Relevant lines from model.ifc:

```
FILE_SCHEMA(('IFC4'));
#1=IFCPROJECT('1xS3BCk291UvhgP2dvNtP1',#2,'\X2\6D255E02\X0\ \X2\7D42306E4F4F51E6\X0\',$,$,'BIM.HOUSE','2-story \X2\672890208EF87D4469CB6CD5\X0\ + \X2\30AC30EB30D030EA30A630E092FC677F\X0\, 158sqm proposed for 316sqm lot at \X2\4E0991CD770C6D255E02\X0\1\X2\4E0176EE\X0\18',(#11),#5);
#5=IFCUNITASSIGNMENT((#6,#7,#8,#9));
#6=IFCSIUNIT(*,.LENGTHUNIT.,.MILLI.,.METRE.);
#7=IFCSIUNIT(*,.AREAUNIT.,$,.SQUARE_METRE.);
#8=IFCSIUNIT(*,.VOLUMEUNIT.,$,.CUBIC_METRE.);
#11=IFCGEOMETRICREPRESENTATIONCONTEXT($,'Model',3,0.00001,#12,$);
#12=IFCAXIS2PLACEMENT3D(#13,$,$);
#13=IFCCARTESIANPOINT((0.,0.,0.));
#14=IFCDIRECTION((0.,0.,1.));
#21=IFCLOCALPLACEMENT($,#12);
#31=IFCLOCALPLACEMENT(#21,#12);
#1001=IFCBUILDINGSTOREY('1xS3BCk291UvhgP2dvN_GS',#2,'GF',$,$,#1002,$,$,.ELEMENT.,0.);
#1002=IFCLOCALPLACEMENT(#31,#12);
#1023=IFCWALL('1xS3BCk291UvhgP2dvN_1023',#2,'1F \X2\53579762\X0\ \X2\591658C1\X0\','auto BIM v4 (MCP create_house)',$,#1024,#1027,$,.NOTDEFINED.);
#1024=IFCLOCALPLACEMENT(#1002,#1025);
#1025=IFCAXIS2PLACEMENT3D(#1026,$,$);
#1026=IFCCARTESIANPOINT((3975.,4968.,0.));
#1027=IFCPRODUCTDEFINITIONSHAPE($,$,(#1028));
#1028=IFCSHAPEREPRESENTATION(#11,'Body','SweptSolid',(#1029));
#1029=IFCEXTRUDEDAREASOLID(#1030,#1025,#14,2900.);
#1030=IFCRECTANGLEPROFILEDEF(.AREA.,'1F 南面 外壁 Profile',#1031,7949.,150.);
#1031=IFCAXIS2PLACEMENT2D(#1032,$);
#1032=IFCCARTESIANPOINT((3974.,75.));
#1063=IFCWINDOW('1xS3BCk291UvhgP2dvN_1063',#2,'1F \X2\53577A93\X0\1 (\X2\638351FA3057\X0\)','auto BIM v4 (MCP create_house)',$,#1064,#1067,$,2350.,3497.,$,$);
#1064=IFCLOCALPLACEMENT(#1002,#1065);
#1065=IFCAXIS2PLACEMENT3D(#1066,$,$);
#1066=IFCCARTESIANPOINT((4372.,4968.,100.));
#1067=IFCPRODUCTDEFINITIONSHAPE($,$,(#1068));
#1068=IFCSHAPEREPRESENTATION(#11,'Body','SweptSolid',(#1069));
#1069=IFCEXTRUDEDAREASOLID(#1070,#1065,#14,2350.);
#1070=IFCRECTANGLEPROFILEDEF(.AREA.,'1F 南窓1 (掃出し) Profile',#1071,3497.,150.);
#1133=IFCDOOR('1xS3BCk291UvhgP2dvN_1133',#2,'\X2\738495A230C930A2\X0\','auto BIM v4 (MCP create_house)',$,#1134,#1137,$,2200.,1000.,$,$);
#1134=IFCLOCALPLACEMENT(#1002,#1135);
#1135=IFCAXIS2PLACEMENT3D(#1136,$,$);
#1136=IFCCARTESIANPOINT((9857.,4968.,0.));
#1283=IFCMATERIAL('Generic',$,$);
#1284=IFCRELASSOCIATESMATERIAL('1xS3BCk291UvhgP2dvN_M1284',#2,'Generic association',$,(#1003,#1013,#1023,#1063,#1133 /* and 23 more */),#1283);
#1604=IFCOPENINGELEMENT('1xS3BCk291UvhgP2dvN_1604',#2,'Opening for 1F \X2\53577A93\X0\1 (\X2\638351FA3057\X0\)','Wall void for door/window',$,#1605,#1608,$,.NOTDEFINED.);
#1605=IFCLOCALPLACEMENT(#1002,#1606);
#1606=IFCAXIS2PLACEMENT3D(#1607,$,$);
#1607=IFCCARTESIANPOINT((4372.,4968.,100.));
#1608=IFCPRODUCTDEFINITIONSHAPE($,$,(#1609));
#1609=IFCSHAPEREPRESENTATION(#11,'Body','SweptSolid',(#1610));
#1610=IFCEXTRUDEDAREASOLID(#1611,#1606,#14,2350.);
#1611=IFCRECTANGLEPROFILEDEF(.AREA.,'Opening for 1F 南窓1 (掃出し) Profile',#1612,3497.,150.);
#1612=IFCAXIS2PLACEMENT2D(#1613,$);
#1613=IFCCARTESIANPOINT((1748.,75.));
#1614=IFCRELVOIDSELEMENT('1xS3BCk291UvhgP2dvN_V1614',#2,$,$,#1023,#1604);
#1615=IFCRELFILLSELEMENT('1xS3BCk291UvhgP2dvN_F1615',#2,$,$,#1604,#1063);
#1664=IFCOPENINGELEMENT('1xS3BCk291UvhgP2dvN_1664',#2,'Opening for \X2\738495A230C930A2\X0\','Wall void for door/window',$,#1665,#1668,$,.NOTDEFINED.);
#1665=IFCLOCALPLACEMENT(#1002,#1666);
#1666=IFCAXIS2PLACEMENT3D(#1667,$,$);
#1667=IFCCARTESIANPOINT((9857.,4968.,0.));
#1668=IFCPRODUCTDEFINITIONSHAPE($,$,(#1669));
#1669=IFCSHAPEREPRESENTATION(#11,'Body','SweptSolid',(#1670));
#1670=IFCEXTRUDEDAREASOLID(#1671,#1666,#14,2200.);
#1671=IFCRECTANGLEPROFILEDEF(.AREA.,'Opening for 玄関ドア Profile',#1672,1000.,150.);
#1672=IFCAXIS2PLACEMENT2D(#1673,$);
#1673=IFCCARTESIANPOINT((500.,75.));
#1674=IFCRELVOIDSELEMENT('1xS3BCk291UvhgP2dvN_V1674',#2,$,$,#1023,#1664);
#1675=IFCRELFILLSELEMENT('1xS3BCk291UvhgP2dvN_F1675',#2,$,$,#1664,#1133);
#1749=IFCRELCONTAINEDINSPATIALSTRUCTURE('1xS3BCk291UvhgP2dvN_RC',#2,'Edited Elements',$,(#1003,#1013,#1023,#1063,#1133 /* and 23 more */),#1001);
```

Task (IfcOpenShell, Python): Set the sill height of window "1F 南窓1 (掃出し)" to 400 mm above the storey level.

```python
import numpy as np
import ifcopenshell
import ifcopenshell.api.geometry
import ifcopenshell.geom
import ifcopenshell.util.element
import ifcopenshell.util.placement
import ifcopenshell.util.shape
import ifcopenshell.util.unit

model = ifcopenshell.open("model.ifc")
unit_scale = ifcopenshell.util.unit.calculate_unit_scale(model)

window = model.by_id(1063)
opening = window.FillsVoids[0].RelatingOpeningElement
storey = ifcopenshell.util.element.get_container(window, ifc_class="IfcBuildingStorey")
level = ifcopenshell.util.placement.get_local_placement(storey.ObjectPlacement)[2, 3]

# The opening's origin need not be at the sill, so measure its lowest point.
shape = ifcopenshell.geom.create_shape(ifcopenshell.geom.settings(), opening)
bottom = ifcopenshell.util.shape.get_shape_bottom_elevation(shape, shape.geometry) / unit_scale
dz = level + 400.0 - bottom

shift = np.array([0.0, 0.0, dz])
# The window is not placed relative to its opening, so move both.
for product in (opening, window):
    matrix = ifcopenshell.util.placement.get_local_placement(product.ObjectPlacement)
    matrix[:3, 3] += shift
    ifcopenshell.api.geometry.edit_object_placement(model, product=product, matrix=matrix, is_si=False)

print(f"moved by {dz * unit_scale:+.3f} m")

model.write("model_rev.ifc")
```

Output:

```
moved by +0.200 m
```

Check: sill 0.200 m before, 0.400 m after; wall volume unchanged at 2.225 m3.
